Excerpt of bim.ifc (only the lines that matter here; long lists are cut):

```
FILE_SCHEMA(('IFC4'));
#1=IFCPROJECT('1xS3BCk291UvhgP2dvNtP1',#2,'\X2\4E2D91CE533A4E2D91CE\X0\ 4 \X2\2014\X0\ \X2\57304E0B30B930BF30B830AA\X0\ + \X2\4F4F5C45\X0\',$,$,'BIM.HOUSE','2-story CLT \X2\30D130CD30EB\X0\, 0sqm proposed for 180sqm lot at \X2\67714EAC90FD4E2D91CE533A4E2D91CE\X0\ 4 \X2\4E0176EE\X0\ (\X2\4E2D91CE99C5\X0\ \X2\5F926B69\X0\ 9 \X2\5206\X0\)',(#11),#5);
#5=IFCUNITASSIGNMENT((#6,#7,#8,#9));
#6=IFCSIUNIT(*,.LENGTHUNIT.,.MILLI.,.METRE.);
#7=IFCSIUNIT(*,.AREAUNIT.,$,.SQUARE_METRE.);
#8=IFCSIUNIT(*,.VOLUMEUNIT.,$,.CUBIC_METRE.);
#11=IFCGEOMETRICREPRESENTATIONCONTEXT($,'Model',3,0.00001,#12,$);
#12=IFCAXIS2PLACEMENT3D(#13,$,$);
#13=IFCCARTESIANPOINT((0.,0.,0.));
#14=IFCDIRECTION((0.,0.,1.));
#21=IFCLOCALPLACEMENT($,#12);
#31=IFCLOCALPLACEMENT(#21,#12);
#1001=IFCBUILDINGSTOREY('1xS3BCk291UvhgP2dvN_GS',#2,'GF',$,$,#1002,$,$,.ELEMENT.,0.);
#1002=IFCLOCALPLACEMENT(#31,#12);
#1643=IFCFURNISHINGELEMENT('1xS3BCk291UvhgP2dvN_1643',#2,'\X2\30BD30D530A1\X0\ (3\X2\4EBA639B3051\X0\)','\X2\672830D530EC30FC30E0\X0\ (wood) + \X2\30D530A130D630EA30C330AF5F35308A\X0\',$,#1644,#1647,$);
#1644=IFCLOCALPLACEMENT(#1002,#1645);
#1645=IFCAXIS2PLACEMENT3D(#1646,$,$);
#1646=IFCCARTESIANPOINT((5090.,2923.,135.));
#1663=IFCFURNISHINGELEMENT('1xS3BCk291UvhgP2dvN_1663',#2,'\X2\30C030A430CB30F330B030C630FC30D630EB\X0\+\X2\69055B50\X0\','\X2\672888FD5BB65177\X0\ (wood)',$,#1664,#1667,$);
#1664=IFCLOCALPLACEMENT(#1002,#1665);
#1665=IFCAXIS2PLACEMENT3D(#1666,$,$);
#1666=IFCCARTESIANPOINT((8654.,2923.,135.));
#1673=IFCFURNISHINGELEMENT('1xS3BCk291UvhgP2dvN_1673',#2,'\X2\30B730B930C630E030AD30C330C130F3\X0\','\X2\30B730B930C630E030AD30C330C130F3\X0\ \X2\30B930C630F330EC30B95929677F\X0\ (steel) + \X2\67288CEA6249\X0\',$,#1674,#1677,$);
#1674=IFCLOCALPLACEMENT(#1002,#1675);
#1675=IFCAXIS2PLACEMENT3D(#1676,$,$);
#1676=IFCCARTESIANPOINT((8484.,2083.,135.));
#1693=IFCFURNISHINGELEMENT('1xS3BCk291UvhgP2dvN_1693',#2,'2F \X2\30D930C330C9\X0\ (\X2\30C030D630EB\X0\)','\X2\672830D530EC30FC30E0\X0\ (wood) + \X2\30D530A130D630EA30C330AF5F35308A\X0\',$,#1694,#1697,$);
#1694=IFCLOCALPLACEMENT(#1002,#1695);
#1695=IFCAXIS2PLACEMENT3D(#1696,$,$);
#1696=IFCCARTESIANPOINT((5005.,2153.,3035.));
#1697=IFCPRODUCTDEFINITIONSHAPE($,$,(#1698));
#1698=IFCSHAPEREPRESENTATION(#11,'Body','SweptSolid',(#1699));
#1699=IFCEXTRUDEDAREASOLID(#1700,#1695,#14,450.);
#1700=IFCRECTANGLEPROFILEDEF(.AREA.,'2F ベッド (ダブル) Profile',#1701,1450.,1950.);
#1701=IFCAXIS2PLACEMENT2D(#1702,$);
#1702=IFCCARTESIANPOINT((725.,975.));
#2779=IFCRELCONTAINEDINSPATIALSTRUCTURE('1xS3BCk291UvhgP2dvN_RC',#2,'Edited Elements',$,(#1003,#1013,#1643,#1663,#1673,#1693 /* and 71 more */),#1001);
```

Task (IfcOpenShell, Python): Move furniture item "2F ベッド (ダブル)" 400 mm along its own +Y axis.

```python
import ifcopenshell
import ifcopenshell.api.geometry
import ifcopenshell.util.placement
import ifcopenshell.util.unit

model = ifcopenshell.open("bim.ifc")
unit_scale = ifcopenshell.util.unit.calculate_unit_scale(model)

item = model.by_guid("1xS3BCk291UvhgP2dvN_1693")
matrix = ifcopenshell.util.placement.get_local_placement(item.ObjectPlacement)
matrix[:3, 3] += matrix[:3, 1] * 0.4 / unit_scale
ifcopenshell.api.geometry.edit_object_placement(model, product=item, matrix=matrix, is_si=False)

print(ifcopenshell.util.placement.get_local_placement(item.ObjectPlacement).round(3) + 0.0)

model.write("bim_rev.ifc")
```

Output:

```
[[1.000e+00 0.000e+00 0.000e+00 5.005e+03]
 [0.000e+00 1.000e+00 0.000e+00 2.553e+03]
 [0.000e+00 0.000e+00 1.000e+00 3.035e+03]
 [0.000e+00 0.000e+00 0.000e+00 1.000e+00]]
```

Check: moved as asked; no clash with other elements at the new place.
